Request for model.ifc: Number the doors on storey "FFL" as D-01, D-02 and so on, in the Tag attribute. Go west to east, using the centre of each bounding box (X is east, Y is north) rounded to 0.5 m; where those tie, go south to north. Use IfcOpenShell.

First a look at what the model holds.

```python
import ifcopenshell
import ifcopenshell.util.element
import ifcopenshell.util.placement

model = ifcopenshell.open("model.ifc")
print(model.schema)
storey = next(s for s in model.by_type("IfcBuildingStorey") if s.Name == "FFL")
doors = [e for e in ifcopenshell.util.element.get_decomposition(storey) if e.is_a("IfcDoor")]
for e in sorted(doors, key=lambda e: e.id()):
    origin = ifcopenshell.util.placement.get_local_placement(e.ObjectPlacement)[:3, 3]
    print(e.id(), e.Tag, e.Name, origin.round(2) + 0.0, sep=" | ")
```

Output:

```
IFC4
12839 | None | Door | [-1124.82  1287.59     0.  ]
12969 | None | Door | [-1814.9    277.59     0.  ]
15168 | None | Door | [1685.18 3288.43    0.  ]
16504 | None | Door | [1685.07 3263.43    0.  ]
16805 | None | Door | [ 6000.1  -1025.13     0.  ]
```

```python
import ifcopenshell
import ifcopenshell.geom
import ifcopenshell.util.element
import ifcopenshell.util.shape

model = ifcopenshell.open("model.ifc")
settings = ifcopenshell.geom.settings()
settings.set("use-world-coords", True)


def centre(element):
    shape = ifcopenshell.geom.create_shape(settings, element)
    return ifcopenshell.util.shape.get_bbox_centroid(shape.geometry)


storey = next(s for s in model.by_type("IfcBuildingStorey") if s.Name == "FFL")
doors = [e for e in ifcopenshell.util.element.get_decomposition(storey) if e.is_a("IfcDoor")]

# Insertion points can sit at a corner or the storey origin, so sort by the geometry (in metres).
centres = {e: centre(e) for e in doors}
doors.sort(key=lambda e: (round(centres[e][0] / 0.5), centres[e][1]))

for i, e in enumerate(doors, start=1):
    number = f"D-{i:02d}"
    e.Tag = number
    print(e.id(), number)

model.write("model_rev.ifc")
```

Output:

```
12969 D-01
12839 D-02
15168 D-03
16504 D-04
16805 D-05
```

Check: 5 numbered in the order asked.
